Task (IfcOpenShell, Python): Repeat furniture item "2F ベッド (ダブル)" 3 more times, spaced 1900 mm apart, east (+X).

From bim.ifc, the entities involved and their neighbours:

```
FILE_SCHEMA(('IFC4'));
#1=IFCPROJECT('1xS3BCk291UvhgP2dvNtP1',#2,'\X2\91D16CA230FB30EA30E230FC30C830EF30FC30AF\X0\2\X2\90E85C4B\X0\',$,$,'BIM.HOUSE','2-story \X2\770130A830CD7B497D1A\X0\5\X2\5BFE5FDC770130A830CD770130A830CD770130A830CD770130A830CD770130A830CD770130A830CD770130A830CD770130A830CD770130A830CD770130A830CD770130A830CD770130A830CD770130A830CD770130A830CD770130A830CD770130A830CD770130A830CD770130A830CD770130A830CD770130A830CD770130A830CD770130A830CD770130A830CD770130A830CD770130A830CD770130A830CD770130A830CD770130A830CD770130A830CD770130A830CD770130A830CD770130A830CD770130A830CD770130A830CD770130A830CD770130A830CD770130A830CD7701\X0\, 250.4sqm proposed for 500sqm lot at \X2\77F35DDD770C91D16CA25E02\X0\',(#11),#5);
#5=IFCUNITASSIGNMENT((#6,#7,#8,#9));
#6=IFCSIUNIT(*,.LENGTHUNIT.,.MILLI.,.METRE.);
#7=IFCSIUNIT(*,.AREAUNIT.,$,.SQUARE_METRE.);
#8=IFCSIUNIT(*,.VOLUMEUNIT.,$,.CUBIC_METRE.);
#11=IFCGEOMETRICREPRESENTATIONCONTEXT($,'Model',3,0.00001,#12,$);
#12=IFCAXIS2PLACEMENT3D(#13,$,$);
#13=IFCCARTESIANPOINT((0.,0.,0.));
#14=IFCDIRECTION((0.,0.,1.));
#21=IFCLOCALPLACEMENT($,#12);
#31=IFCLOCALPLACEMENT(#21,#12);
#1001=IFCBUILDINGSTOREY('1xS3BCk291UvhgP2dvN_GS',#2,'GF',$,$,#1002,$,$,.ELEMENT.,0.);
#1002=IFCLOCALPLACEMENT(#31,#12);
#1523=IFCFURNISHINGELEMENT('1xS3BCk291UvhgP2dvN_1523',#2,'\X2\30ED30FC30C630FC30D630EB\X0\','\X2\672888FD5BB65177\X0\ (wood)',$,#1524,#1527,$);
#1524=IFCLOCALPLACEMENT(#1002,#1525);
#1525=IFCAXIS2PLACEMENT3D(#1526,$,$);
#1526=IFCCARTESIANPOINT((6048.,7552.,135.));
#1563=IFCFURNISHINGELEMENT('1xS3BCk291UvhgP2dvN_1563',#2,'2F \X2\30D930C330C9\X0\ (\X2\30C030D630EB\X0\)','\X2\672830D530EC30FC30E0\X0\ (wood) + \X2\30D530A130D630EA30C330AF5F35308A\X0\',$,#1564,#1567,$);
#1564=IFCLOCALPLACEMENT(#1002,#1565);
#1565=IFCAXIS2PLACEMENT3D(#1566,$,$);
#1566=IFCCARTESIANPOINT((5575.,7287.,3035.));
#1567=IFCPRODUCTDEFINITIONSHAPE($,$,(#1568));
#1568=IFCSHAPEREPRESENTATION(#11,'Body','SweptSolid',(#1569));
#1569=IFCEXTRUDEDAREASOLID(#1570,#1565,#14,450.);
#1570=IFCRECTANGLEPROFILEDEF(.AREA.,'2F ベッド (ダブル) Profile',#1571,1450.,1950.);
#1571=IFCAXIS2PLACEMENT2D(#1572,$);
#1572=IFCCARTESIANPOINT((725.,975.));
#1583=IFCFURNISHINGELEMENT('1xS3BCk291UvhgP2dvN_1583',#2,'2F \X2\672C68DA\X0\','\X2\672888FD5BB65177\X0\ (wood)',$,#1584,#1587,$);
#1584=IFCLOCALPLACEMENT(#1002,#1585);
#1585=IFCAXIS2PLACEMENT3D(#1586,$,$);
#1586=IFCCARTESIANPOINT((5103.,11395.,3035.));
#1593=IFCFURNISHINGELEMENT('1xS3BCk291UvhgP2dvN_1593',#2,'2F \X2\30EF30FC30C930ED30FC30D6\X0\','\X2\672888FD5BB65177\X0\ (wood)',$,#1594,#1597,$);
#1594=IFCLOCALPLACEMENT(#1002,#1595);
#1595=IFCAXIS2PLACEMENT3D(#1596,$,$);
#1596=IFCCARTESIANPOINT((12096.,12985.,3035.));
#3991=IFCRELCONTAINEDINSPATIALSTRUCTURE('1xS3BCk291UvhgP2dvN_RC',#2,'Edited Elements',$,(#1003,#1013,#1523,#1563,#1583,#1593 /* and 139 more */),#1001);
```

```python
import numpy as np
import ifcopenshell
import ifcopenshell.api.geometry
import ifcopenshell.api.root
import ifcopenshell.util.element
import ifcopenshell.util.placement
import ifcopenshell.util.unit

model = ifcopenshell.open("bim.ifc")
unit_scale = ifcopenshell.util.unit.calculate_unit_scale(model)


def reuse_history(source, copy):
    """copy_class also copies each property set's owner history, people and application; keep the originals."""
    for rel in copy.IsDefinedBy:
        if rel.is_a("IfcRelDefinesByProperties") and (history := rel.RelatingPropertyDefinition.OwnerHistory):
            rel.RelatingPropertyDefinition.OwnerHistory = source.OwnerHistory
            ifcopenshell.util.element.remove_deep2(model, history)


source = model.by_id(1563)
base = ifcopenshell.util.placement.get_local_placement(source.ObjectPlacement)
step = np.array([1.0, 0.0, 0.0]) * 1.9 / unit_scale

for i in range(1, 4):
    copy = ifcopenshell.api.root.copy_class(model, product=source)
    copy.Representation = ifcopenshell.util.element.copy_deep(
        model, source.Representation, exclude=["IfcGeometricRepresentationContext", "IfcRepresentationMap"]
    )
    reuse_history(source, copy)
    matrix = base.copy()
    matrix[:3, 3] += i * step
    print("added at", matrix[:3, 3].round(3) + 0.0)
    ifcopenshell.api.geometry.edit_object_placement(model, product=copy, matrix=matrix, is_si=False)

model.write("bim-out.ifc")
```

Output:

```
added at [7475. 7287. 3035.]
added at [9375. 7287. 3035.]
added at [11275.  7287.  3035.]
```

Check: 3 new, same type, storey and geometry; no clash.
